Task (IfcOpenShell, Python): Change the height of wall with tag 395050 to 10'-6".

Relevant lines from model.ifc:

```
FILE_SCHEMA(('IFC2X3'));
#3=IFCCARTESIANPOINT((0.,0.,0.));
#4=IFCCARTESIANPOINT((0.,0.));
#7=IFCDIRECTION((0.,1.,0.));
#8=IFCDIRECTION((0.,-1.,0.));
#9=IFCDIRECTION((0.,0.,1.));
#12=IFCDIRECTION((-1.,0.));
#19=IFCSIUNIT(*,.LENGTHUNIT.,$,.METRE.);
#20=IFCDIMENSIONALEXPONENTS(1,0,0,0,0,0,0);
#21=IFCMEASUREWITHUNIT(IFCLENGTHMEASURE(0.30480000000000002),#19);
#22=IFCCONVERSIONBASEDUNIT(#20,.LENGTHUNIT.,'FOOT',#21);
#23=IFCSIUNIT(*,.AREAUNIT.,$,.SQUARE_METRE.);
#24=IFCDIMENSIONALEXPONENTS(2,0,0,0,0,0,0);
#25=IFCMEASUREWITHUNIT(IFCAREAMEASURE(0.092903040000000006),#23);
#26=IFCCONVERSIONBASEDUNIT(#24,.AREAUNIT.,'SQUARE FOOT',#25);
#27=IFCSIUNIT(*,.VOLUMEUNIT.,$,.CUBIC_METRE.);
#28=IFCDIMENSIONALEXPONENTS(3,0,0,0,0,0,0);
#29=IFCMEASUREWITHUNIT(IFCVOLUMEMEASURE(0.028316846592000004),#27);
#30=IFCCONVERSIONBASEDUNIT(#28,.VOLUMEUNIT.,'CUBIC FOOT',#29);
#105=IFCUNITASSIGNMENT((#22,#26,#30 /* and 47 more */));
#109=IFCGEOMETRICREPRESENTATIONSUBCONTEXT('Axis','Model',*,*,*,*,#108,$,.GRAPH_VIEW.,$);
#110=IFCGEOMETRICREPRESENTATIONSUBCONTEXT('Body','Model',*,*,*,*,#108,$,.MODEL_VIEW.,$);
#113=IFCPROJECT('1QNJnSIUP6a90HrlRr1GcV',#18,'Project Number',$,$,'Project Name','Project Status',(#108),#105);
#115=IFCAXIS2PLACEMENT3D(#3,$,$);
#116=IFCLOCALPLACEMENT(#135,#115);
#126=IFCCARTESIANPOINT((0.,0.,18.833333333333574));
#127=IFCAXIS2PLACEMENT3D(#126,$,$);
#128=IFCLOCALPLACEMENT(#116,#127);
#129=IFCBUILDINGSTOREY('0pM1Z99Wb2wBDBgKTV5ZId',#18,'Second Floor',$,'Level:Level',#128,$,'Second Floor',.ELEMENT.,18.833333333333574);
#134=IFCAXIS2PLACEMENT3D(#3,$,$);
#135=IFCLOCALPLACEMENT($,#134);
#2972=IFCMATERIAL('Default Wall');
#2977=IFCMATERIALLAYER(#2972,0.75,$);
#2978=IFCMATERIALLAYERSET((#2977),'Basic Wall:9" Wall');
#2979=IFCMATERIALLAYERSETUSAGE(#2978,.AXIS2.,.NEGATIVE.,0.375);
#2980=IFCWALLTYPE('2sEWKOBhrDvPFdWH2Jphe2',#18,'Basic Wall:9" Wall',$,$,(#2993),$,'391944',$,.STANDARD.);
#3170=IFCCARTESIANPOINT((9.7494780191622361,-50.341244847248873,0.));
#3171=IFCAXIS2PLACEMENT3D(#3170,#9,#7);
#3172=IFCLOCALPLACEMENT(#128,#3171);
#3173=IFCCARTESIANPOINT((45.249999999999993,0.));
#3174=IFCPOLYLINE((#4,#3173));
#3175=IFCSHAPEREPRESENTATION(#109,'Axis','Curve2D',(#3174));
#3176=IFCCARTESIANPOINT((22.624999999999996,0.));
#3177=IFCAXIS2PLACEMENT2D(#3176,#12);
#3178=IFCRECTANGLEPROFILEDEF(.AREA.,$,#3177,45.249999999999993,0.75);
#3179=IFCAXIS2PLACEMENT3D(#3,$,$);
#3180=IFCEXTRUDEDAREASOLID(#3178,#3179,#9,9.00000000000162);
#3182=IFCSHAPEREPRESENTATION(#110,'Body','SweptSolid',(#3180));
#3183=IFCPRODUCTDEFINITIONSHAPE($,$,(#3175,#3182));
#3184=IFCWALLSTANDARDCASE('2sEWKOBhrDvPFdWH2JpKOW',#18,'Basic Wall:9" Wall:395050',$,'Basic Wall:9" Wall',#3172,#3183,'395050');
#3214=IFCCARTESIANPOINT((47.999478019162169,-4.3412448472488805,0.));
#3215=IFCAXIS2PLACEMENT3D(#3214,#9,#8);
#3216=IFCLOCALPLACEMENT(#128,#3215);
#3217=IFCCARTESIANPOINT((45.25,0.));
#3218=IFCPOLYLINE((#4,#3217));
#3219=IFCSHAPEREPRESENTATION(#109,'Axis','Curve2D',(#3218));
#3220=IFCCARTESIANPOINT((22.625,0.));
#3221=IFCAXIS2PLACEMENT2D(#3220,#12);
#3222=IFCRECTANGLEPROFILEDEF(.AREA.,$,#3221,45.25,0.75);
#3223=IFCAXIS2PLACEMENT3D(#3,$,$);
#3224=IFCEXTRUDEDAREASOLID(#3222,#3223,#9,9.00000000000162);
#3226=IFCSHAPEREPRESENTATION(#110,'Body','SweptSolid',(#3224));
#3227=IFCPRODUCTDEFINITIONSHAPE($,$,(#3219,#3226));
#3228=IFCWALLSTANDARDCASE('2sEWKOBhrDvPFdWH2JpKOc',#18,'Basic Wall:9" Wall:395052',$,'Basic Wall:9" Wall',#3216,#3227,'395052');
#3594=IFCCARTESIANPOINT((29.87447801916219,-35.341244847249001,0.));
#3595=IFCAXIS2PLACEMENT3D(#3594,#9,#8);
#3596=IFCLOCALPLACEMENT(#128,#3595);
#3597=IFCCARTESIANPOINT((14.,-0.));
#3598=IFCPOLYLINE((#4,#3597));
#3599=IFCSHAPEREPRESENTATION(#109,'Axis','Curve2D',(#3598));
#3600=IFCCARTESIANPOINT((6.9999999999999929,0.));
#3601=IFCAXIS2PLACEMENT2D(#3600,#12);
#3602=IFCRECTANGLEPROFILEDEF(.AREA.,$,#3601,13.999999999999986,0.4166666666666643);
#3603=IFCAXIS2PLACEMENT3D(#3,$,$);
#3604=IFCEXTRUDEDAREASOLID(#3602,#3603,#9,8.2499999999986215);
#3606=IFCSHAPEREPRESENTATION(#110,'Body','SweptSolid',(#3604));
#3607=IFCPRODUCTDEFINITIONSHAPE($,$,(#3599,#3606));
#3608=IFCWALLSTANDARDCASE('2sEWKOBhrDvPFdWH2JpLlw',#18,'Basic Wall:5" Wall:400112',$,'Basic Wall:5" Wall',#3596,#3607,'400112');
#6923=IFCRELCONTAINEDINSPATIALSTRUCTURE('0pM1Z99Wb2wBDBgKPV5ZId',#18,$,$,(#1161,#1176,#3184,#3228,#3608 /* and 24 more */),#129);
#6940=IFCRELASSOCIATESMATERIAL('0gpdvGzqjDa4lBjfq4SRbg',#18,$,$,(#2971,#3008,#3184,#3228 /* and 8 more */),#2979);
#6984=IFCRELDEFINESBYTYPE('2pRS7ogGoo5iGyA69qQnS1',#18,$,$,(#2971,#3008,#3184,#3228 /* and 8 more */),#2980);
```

```python
import ifcopenshell
import ifcopenshell.geom
import ifcopenshell.util.representation
import ifcopenshell.util.shape
import ifcopenshell.util.unit

model = ifcopenshell.open("model.ifc")
unit_scale = ifcopenshell.util.unit.calculate_unit_scale(model)
settings = ifcopenshell.geom.settings()


def volume(element):
    """Net volume in cubic metres, openings subtracted."""
    shape = ifcopenshell.geom.create_shape(settings, element)
    return ifcopenshell.util.shape.get_volume(shape.geometry)


wall = model.by_guid("2sEWKOBhrDvPFdWH2JpKOW")
before = volume(wall)

body = ifcopenshell.util.representation.get_representation(wall, "Model", "Body")
solid = body.Items[0]
old_height = solid.Depth
solid.Depth = 126 * 0.0254 / unit_scale
after = volume(wall)

print(f"height {old_height:g} -> {solid.Depth:g}, volume {before:.3f} -> {after:.3f} m3")

model.write("model-out.ifc")
```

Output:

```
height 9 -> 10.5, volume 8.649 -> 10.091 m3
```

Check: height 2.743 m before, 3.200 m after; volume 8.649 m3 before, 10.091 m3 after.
